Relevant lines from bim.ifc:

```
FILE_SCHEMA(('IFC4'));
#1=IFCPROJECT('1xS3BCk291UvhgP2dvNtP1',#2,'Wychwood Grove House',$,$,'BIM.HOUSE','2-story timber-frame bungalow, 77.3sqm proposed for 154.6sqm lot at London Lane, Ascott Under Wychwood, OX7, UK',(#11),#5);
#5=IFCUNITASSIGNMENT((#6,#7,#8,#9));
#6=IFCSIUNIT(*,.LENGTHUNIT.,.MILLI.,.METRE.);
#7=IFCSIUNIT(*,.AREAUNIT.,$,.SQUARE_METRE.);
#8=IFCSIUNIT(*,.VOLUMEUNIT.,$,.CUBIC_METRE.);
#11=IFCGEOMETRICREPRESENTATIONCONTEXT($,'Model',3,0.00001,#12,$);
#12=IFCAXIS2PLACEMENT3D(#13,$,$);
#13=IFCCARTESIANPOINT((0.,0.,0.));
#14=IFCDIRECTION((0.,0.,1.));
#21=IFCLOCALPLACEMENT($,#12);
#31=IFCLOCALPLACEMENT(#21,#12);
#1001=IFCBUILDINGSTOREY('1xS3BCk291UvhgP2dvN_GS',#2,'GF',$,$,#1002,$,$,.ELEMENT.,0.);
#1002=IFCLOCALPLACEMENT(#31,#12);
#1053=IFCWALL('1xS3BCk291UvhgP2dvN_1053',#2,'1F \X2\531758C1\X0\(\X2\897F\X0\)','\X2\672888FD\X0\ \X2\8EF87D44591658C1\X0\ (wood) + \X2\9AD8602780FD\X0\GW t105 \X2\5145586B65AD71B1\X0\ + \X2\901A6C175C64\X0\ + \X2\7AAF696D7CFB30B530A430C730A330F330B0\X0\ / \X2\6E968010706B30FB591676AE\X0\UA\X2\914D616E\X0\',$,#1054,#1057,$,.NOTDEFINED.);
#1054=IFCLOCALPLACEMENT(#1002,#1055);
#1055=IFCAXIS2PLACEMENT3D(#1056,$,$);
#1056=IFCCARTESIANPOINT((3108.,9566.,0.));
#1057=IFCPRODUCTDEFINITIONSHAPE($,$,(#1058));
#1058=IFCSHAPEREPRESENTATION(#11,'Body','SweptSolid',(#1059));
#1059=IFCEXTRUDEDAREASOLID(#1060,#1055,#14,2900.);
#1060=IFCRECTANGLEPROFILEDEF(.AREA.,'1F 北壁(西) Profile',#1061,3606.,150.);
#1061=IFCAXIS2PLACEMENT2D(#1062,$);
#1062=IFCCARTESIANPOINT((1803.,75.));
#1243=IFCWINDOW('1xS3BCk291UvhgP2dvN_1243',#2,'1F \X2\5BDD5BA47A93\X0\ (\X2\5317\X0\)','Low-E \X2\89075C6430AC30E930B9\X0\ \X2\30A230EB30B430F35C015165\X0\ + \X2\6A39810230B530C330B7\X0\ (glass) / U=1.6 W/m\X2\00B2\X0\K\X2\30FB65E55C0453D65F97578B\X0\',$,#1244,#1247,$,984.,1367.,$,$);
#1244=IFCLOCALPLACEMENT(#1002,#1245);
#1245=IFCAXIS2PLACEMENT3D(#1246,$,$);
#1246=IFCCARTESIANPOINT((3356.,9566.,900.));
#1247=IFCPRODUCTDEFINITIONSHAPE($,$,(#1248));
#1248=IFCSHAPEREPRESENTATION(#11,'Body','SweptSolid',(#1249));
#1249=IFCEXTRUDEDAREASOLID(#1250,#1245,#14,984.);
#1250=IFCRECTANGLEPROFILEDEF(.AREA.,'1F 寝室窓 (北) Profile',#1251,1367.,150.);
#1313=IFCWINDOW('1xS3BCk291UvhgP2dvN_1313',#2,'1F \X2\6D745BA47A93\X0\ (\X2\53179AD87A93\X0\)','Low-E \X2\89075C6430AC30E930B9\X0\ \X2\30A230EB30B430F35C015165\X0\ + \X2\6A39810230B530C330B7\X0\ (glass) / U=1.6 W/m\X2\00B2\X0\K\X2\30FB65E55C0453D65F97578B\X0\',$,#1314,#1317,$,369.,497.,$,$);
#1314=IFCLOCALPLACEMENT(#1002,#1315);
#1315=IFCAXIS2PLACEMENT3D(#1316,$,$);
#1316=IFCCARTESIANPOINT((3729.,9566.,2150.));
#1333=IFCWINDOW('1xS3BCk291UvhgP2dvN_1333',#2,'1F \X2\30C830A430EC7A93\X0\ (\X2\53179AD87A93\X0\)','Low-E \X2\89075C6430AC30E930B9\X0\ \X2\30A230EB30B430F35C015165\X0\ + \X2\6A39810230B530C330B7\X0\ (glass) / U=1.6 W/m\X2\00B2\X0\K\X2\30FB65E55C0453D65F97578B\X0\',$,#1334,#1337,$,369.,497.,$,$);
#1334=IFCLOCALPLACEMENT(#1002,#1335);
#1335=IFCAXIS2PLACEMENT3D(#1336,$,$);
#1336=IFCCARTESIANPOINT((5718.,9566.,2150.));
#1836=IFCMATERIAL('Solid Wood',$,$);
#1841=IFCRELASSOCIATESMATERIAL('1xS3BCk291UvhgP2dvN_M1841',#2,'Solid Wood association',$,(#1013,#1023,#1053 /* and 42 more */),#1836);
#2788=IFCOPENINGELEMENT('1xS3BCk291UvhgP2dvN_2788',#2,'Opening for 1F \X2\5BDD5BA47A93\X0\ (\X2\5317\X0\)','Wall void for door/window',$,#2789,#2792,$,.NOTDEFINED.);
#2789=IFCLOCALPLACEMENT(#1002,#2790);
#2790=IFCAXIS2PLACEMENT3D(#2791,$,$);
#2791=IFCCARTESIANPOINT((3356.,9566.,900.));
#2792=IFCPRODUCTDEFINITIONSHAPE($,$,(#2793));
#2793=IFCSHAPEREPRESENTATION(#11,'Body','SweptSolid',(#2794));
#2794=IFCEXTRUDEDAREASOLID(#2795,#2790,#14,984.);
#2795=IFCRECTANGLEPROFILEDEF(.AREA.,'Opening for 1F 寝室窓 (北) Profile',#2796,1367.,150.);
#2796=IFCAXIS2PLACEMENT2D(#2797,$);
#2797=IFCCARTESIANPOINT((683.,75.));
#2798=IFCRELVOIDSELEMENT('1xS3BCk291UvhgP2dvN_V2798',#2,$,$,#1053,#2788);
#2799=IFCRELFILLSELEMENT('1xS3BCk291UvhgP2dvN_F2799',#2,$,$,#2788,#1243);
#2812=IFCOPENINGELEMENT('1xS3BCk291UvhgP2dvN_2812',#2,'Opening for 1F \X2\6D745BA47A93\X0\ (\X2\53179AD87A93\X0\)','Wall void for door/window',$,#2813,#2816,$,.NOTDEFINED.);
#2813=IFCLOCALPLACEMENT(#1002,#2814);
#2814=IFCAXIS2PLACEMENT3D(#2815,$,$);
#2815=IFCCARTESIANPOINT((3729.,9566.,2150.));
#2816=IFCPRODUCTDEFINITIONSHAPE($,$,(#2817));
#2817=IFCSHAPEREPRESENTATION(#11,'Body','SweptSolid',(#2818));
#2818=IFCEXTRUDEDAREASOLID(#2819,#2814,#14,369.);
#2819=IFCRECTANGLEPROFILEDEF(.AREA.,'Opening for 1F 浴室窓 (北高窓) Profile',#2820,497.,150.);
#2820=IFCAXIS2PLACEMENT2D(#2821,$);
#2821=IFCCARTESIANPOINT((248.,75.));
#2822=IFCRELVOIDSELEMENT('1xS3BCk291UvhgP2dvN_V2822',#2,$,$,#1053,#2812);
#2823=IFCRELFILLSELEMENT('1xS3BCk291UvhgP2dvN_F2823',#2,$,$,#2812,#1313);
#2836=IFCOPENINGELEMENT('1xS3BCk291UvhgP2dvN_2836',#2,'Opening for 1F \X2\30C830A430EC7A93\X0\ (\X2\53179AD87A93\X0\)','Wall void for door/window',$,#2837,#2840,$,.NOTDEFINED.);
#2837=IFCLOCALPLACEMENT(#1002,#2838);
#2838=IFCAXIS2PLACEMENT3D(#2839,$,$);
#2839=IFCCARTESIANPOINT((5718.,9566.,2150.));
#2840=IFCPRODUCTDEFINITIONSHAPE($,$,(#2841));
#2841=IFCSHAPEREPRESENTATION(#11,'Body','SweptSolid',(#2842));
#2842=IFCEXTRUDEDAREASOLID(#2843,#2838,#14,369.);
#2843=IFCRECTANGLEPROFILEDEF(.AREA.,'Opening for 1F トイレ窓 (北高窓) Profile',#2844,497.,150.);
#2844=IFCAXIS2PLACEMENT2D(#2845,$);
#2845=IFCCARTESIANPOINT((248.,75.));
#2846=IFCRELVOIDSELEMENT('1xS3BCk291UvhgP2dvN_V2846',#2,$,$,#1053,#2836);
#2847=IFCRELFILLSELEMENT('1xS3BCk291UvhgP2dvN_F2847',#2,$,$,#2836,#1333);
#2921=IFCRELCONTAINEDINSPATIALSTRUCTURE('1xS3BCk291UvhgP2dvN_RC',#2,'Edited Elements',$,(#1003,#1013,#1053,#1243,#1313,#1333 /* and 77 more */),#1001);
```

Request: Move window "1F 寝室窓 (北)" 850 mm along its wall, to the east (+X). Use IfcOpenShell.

```python
import ifcopenshell
import ifcopenshell.api.geometry
import ifcopenshell.util.placement

model = ifcopenshell.open("bim.ifc")

window = model.by_guid("1xS3BCk291UvhgP2dvN_1243")
opening = window.FillsVoids[0].RelatingOpeningElement
wall = opening.VoidsElements[0].RelatingBuildingElement

wall_matrix = ifcopenshell.util.placement.get_local_placement(wall.ObjectPlacement)
shift = wall_matrix[:3, 0] * 850.0
before = ifcopenshell.util.placement.get_local_placement(window.ObjectPlacement)[:3, 3].copy()

# The window is not placed relative to its opening, so move both.
for product in (opening, window):
    matrix = ifcopenshell.util.placement.get_local_placement(product.ObjectPlacement)
    matrix[:3, 3] += shift
    ifcopenshell.api.geometry.edit_object_placement(model, product=product, matrix=matrix, is_si=False)

after = ifcopenshell.util.placement.get_local_placement(window.ObjectPlacement)[:3, 3]
print("window moved by", (after - before).round(3) + 0.0)

model.write("bim_updated.ifc")
```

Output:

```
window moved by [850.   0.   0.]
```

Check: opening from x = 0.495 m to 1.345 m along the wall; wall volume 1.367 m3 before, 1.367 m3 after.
